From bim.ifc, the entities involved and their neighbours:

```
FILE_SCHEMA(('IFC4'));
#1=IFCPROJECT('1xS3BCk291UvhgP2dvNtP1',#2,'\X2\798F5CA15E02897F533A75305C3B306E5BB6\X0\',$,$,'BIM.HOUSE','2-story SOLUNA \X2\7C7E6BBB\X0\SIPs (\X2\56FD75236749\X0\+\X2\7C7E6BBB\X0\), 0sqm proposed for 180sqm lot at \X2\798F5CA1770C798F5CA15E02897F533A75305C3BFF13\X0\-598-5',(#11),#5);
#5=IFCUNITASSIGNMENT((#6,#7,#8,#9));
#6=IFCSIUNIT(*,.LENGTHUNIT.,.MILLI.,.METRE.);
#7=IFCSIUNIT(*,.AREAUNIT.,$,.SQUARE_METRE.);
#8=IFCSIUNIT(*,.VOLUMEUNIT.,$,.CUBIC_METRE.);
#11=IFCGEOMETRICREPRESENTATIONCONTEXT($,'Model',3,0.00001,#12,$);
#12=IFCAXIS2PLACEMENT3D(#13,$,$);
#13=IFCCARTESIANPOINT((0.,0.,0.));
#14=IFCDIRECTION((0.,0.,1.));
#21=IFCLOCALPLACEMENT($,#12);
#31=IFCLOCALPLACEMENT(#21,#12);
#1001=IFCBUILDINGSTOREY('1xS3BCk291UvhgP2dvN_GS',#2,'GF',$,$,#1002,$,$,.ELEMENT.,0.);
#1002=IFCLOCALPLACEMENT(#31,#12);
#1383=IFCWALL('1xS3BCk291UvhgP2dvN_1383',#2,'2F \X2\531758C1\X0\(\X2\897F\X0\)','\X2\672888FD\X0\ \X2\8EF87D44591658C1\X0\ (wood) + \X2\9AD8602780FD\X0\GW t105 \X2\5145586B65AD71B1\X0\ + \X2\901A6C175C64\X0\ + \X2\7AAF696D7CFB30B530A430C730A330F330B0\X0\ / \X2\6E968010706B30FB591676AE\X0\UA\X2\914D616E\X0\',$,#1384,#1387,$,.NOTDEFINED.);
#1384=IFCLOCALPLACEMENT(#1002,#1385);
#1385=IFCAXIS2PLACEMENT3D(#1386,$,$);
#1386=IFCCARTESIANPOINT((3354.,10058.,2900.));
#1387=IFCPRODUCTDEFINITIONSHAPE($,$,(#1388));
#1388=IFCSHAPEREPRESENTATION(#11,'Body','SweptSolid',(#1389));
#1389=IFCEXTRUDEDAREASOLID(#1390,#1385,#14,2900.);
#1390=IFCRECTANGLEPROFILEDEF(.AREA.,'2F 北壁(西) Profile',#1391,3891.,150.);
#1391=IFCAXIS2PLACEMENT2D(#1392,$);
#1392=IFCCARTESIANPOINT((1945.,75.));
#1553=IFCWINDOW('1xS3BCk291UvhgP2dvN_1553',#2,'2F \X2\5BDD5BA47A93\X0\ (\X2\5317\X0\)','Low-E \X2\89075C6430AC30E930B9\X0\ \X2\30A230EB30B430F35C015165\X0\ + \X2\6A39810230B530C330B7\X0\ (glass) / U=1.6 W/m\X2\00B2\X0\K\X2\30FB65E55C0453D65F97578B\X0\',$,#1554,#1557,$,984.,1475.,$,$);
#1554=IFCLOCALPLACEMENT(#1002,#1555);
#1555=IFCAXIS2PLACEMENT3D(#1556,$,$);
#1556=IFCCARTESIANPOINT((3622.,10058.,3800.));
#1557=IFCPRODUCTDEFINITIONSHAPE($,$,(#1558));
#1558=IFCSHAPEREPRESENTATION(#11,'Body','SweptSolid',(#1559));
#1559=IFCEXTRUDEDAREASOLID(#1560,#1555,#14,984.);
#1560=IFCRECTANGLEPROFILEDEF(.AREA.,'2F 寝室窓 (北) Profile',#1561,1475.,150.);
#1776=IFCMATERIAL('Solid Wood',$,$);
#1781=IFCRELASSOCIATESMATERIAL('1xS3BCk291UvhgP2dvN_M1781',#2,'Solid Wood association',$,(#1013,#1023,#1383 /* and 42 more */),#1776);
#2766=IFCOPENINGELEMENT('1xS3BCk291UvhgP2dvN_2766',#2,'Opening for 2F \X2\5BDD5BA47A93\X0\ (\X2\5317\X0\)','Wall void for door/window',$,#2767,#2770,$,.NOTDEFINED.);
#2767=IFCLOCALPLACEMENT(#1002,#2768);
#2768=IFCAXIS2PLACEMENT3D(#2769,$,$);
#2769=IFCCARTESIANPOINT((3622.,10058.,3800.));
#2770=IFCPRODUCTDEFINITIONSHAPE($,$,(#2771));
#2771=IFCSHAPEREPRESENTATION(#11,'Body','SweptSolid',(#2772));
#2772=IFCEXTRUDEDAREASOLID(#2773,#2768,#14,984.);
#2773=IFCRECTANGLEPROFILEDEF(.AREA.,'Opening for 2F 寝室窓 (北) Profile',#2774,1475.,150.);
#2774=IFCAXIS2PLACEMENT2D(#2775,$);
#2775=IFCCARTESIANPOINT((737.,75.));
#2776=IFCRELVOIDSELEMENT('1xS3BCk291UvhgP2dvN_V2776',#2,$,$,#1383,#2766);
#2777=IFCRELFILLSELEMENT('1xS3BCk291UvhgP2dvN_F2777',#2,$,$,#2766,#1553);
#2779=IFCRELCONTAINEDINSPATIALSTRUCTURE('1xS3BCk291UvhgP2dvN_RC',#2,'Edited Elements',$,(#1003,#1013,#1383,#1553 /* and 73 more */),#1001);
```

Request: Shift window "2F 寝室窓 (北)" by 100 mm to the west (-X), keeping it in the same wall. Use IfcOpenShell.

```python
import ifcopenshell
import ifcopenshell.api.geometry
import ifcopenshell.util.placement
import ifcopenshell.util.unit

model = ifcopenshell.open("bim.ifc")
unit_scale = ifcopenshell.util.unit.calculate_unit_scale(model)

window = model.by_guid("1xS3BCk291UvhgP2dvN_1553")
opening = window.FillsVoids[0].RelatingOpeningElement
wall = opening.VoidsElements[0].RelatingBuildingElement

wall_matrix = ifcopenshell.util.placement.get_local_placement(wall.ObjectPlacement)
shift = wall_matrix[:3, 0] * -0.1 / unit_scale
before = ifcopenshell.util.placement.get_local_placement(window.ObjectPlacement)[:3, 3].copy()

# The window is not placed relative to its opening, so move both.
for product in (opening, window):
    matrix = ifcopenshell.util.placement.get_local_placement(product.ObjectPlacement)
    matrix[:3, 3] += shift
    ifcopenshell.api.geometry.edit_object_placement(model, product=product, matrix=matrix, is_si=False)

after = ifcopenshell.util.placement.get_local_placement(window.ObjectPlacement)[:3, 3]
print("window moved by", (after - before).round(3) + 0.0)

model.write("bim_edited.ifc")
```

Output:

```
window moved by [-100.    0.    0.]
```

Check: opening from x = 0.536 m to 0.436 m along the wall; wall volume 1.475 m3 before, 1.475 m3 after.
